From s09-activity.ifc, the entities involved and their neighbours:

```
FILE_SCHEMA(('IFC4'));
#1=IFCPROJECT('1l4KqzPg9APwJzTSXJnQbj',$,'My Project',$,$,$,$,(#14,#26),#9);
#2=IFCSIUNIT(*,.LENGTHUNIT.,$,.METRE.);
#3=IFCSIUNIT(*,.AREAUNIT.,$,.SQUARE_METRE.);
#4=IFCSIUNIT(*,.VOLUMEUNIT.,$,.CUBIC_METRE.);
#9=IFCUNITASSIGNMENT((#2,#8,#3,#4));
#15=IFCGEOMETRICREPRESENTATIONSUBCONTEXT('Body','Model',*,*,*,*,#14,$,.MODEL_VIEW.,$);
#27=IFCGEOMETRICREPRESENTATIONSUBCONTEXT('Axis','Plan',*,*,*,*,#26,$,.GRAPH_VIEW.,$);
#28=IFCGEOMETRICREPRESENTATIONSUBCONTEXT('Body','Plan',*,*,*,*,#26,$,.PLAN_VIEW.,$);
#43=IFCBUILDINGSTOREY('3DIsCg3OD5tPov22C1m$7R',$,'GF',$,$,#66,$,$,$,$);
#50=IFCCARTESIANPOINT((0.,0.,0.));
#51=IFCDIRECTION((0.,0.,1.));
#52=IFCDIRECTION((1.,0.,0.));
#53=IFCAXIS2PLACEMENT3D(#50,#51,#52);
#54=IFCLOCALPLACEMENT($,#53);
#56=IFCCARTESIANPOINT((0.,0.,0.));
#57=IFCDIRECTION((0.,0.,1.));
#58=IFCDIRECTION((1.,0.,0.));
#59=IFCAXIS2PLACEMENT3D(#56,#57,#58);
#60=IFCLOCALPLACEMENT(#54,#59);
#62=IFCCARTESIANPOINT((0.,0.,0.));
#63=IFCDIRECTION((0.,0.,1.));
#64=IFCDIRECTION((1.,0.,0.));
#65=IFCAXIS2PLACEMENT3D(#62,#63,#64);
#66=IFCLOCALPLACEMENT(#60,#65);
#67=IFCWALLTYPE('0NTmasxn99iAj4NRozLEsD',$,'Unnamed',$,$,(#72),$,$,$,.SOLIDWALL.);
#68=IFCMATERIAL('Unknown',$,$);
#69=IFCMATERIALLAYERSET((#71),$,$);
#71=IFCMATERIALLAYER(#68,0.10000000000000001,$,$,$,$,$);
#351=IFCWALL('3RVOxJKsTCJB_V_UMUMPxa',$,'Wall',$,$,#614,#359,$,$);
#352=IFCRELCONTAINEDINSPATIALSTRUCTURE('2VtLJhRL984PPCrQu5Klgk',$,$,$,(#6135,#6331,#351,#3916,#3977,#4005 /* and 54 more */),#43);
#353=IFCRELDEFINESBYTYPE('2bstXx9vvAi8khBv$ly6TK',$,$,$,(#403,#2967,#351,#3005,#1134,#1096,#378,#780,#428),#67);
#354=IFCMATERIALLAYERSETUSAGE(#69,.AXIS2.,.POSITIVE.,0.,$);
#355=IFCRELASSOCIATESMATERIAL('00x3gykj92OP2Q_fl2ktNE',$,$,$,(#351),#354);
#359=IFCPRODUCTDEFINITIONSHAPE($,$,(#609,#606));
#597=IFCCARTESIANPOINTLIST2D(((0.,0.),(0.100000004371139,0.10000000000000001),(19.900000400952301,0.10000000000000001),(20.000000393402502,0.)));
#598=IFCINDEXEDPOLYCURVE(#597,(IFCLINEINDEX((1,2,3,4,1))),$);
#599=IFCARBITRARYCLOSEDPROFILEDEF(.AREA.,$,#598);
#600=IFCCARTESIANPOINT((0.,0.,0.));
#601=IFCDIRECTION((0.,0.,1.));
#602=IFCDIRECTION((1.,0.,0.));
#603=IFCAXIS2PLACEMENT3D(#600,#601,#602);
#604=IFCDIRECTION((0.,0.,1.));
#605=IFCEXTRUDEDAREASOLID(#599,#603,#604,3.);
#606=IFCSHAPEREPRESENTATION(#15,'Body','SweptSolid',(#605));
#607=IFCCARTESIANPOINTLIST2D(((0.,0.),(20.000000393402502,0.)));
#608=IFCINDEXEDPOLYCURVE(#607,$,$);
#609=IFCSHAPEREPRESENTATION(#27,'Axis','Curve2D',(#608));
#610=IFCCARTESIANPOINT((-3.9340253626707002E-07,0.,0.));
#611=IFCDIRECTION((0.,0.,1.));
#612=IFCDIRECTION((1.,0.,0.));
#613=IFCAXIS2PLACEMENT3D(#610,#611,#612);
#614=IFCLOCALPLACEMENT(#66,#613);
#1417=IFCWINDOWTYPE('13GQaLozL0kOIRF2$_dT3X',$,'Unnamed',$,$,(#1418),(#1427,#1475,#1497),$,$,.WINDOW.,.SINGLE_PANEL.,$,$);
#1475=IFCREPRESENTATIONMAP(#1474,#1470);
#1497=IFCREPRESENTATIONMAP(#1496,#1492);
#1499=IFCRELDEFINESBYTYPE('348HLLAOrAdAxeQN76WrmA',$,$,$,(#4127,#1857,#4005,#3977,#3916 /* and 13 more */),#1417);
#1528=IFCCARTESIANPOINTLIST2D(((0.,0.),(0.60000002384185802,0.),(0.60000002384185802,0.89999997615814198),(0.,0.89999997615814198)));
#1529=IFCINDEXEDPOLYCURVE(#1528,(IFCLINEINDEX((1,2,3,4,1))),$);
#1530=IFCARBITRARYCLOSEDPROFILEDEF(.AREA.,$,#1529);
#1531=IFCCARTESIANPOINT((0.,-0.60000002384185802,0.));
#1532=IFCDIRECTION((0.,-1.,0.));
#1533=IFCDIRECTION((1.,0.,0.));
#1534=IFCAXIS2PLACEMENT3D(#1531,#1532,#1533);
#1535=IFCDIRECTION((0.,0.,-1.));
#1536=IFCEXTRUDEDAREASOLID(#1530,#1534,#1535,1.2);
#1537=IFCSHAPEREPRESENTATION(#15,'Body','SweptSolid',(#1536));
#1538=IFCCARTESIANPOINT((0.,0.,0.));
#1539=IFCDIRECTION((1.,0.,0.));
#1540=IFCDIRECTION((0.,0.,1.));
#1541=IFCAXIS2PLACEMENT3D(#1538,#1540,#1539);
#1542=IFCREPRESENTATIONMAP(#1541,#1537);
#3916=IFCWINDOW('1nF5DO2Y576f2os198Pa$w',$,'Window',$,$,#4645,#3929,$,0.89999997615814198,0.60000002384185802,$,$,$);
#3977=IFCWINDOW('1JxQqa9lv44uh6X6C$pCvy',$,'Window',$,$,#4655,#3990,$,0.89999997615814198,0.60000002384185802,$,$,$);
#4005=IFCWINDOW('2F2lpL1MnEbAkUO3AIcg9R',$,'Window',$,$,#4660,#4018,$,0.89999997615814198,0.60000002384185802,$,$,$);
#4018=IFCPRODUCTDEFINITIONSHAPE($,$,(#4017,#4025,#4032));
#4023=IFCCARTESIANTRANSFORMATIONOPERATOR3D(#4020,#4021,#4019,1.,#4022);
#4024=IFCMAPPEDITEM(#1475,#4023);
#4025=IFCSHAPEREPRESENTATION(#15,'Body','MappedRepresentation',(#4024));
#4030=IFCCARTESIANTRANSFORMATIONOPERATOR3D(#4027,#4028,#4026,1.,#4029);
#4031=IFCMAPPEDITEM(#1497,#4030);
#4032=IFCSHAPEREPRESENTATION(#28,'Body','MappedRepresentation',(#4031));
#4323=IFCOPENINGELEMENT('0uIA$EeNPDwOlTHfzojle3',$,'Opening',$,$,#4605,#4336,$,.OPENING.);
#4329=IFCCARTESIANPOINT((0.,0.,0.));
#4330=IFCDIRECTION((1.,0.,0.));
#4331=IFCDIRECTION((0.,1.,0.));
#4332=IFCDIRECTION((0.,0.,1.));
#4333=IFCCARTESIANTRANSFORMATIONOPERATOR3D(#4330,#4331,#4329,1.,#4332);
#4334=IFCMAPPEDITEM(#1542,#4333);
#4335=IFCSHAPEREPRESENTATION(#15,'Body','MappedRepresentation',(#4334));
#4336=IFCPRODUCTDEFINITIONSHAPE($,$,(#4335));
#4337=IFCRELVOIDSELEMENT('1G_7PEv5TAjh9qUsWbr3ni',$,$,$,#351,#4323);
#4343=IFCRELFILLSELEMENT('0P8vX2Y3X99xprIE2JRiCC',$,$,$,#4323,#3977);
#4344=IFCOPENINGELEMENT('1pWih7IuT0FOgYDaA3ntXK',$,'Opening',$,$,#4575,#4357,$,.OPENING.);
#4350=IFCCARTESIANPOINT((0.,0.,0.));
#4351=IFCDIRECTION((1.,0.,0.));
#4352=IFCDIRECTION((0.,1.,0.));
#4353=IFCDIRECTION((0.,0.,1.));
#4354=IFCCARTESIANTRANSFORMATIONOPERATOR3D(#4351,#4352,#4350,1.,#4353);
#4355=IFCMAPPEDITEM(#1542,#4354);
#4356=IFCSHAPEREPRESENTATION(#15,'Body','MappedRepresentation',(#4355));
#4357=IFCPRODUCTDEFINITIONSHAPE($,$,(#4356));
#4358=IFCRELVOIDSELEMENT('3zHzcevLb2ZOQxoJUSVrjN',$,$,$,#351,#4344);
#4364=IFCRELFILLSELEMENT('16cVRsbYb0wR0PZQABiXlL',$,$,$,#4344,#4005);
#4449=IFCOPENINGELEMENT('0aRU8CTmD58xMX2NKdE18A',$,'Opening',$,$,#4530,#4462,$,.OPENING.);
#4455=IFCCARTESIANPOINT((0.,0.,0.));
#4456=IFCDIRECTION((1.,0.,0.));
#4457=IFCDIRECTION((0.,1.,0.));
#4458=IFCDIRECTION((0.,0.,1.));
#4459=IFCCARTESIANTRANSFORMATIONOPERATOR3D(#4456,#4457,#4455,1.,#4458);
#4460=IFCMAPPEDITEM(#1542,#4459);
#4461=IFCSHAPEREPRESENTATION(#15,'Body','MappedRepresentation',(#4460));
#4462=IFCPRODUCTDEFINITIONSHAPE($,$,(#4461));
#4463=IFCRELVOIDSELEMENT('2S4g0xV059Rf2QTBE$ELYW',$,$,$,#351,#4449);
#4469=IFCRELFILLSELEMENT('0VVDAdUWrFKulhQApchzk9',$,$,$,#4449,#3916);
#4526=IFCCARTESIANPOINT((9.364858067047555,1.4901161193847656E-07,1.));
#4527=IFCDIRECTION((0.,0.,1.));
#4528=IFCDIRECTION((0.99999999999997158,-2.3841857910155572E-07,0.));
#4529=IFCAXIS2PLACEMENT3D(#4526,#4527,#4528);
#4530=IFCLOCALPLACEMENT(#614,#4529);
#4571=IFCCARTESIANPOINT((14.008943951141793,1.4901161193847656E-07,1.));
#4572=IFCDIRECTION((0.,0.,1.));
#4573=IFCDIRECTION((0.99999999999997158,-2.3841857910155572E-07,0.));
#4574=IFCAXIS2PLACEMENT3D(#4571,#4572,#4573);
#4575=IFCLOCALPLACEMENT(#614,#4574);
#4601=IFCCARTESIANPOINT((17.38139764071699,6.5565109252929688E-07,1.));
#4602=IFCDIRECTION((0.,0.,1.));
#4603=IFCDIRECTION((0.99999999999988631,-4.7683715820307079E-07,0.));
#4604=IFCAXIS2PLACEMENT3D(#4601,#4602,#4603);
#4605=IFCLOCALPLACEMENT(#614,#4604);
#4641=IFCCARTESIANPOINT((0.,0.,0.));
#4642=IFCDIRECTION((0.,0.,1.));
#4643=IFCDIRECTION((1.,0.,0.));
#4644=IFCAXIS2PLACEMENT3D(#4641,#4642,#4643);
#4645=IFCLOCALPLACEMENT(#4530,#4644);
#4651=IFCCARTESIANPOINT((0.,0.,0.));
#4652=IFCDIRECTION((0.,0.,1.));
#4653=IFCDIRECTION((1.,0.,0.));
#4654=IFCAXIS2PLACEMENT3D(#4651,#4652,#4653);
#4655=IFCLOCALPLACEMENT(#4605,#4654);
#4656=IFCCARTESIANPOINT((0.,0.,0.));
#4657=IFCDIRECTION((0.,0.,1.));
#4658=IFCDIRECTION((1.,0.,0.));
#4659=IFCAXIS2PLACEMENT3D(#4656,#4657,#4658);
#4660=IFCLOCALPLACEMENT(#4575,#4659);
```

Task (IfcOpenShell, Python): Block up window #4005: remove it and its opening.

```python
import ifcopenshell
import ifcopenshell.api.feature
import ifcopenshell.api.root
import ifcopenshell.geom
import ifcopenshell.util.shape

model = ifcopenshell.open("s09-activity.ifc")
settings = ifcopenshell.geom.settings()


def volume(element):
    """Net volume in cubic metres, openings subtracted."""
    shape = ifcopenshell.geom.create_shape(settings, element)
    return ifcopenshell.util.shape.get_volume(shape.geometry)


window = model.by_id(4005)
opening = window.FillsVoids[0].RelatingOpeningElement
wall = opening.VoidsElements[0].RelatingBuildingElement
before = volume(wall)

ifcopenshell.api.root.remove_product(model, product=window)
ifcopenshell.api.feature.remove_feature(model, feature=opening)

after = volume(wall)

print(f"wall volume {before:.3f} -> {after:.3f} m3")

model.write("s09-activity_rev.ifc")
```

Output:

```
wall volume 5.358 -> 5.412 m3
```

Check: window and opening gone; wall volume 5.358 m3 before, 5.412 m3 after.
